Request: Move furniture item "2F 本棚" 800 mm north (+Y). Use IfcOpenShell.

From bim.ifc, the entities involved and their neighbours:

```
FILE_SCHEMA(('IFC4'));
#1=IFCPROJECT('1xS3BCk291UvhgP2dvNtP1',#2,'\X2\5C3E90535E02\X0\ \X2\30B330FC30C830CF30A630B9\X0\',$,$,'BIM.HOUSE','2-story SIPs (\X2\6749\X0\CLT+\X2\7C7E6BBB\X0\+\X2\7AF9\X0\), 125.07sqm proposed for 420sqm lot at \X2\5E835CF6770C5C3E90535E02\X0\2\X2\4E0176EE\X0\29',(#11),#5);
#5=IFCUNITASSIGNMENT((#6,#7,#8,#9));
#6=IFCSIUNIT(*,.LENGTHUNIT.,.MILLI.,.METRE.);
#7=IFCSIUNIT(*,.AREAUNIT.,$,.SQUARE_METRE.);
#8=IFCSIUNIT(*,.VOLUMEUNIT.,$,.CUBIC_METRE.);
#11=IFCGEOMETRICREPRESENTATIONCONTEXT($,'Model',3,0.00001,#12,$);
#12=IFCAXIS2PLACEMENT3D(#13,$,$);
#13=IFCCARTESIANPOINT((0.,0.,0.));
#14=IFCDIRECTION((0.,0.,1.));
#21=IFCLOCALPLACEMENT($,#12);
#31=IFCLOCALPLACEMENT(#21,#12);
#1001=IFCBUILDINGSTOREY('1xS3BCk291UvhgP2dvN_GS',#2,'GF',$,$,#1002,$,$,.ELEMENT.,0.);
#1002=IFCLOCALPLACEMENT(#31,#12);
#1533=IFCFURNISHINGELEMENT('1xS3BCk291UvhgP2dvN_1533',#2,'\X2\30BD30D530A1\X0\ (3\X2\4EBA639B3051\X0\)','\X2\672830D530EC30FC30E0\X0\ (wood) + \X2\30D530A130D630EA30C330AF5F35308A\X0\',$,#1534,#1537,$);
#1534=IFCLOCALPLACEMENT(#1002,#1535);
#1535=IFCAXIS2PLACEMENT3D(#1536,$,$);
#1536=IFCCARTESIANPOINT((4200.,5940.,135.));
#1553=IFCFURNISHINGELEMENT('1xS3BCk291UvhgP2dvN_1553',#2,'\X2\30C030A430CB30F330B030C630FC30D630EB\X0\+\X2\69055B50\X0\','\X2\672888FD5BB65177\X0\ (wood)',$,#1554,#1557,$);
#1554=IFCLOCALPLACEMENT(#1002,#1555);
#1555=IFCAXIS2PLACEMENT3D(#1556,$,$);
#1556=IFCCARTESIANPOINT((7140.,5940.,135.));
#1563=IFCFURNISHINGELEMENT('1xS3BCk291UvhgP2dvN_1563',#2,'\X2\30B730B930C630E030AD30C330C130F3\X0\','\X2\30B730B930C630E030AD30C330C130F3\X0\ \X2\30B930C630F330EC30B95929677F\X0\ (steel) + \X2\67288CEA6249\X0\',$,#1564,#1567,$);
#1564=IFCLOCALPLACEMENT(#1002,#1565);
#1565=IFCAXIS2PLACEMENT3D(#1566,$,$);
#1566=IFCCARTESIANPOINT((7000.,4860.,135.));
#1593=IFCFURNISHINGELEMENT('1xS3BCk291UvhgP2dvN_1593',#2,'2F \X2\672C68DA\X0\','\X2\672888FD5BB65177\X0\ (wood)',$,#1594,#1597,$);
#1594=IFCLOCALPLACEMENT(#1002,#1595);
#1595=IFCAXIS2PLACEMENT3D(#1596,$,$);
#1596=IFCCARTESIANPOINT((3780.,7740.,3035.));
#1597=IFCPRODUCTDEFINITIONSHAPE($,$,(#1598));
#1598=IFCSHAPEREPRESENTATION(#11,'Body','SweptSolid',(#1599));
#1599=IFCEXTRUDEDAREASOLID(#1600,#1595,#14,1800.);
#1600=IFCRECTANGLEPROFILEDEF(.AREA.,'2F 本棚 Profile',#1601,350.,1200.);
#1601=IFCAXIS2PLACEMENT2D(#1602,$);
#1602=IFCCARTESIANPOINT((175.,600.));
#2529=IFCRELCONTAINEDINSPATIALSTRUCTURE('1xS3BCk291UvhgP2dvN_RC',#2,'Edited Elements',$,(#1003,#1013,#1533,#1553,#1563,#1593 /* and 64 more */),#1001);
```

```python
import ifcopenshell
import ifcopenshell.api.geometry
import ifcopenshell.util.placement

model = ifcopenshell.open("bim.ifc")

item = model.by_id(1593)
matrix = ifcopenshell.util.placement.get_local_placement(item.ObjectPlacement)
matrix[1, 3] += 800.0
ifcopenshell.api.geometry.edit_object_placement(model, product=item, matrix=matrix, is_si=False)

print(ifcopenshell.util.placement.get_local_placement(item.ObjectPlacement).round(3) + 0.0)

model.write("bim_updated.ifc")
```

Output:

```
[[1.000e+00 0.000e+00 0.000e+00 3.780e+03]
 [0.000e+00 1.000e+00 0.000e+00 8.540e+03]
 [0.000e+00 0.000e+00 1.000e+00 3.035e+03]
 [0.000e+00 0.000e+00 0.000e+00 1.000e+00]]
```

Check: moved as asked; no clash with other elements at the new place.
